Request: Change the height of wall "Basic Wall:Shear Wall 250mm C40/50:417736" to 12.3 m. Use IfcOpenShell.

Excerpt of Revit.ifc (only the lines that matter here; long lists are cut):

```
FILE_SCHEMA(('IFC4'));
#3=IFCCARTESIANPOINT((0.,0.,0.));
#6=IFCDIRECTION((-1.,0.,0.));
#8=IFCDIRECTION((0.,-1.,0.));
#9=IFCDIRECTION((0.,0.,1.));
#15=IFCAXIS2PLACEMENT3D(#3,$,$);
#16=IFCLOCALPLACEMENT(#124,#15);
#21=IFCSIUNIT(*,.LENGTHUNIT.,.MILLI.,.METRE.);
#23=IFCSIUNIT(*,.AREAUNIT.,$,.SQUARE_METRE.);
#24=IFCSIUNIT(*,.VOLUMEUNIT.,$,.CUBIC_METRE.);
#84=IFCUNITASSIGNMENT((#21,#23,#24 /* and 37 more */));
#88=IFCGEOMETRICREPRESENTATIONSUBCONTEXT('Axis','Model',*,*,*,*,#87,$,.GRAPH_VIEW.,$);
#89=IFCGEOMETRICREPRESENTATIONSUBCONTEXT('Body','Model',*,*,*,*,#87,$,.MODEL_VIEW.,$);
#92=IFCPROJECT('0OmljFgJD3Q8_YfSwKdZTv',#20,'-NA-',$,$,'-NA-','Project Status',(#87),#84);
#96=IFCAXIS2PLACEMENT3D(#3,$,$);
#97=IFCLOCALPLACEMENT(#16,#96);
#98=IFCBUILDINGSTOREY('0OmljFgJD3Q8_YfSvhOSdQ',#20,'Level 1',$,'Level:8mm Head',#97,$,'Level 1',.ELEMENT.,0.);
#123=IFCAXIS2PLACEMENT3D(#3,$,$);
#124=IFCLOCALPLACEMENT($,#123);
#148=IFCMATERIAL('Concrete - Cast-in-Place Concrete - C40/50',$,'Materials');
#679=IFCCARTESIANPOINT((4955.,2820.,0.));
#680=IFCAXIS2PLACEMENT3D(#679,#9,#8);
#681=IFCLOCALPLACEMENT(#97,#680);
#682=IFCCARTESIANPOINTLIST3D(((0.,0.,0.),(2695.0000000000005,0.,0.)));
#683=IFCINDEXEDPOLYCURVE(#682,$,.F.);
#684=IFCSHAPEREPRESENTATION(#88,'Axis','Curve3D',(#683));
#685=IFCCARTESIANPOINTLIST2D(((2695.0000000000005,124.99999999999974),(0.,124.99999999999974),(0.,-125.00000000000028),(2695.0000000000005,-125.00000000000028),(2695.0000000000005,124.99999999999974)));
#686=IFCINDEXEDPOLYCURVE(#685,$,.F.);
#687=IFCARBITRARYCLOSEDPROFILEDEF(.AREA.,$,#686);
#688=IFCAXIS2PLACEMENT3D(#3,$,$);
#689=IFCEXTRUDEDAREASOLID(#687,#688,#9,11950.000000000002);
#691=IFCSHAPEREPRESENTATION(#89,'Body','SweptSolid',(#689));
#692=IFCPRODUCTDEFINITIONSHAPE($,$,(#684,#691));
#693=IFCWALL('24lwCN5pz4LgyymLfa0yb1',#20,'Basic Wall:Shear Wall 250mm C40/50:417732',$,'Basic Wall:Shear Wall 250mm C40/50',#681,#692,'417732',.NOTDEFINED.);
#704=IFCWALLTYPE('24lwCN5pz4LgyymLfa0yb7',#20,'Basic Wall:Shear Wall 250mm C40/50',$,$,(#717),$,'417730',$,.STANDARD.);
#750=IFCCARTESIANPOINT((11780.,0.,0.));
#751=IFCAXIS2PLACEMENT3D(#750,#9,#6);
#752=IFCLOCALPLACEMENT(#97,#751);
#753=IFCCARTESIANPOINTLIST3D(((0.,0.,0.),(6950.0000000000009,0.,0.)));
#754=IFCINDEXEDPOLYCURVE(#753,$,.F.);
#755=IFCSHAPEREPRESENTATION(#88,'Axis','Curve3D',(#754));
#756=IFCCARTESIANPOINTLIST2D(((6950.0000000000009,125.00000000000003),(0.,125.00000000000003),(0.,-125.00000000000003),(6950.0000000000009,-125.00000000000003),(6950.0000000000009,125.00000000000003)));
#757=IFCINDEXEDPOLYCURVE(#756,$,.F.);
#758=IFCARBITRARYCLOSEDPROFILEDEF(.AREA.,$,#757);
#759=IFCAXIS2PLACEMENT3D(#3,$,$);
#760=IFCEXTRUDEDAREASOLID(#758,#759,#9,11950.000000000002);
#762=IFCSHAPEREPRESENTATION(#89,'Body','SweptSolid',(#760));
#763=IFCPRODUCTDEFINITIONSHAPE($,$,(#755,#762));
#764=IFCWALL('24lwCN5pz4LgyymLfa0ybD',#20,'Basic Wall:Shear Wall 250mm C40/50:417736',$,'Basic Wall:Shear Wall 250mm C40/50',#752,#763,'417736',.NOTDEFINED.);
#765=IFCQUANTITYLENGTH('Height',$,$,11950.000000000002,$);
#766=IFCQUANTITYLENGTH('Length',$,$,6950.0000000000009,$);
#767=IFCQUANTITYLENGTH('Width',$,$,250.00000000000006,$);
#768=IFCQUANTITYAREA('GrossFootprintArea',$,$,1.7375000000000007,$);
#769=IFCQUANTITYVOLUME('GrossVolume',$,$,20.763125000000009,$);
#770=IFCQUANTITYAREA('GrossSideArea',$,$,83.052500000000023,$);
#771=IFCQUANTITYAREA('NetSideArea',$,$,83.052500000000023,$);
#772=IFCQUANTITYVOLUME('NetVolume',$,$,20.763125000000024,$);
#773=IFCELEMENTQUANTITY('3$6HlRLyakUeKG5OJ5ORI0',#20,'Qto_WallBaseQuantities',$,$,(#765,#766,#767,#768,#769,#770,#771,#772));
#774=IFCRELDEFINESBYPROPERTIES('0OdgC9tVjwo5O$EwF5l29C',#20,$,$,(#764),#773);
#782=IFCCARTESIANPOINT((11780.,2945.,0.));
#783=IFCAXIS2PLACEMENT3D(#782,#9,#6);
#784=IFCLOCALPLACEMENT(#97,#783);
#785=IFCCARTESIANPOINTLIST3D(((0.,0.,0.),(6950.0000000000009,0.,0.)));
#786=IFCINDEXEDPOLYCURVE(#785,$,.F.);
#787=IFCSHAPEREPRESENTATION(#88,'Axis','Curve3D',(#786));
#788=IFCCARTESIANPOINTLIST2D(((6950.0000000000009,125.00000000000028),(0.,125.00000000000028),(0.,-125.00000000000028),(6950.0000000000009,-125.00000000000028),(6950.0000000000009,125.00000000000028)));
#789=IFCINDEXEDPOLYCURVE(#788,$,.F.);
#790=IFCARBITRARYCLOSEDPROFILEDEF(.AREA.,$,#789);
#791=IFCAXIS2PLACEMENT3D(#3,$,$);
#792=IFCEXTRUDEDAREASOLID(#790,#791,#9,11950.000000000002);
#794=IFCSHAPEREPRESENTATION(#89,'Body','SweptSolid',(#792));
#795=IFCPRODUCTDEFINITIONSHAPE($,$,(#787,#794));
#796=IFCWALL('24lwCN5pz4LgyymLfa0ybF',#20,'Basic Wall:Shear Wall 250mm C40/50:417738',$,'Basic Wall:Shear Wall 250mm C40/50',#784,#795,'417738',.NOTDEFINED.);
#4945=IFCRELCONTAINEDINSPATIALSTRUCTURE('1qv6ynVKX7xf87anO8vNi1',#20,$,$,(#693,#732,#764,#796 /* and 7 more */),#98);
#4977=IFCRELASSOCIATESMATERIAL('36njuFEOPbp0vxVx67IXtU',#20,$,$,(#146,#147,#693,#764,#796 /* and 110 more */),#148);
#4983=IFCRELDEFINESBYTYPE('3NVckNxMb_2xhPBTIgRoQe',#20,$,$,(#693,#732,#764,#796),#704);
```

```python
import ifcopenshell
import ifcopenshell.api.pset
import ifcopenshell.geom
import ifcopenshell.util.element
import ifcopenshell.util.representation
import ifcopenshell.util.shape
import ifcopenshell.util.unit

model = ifcopenshell.open("Revit.ifc")
unit_scale = ifcopenshell.util.unit.calculate_unit_scale(model)
area_scale = ifcopenshell.util.unit.calculate_unit_scale(model, "AREAUNIT")
volume_scale = ifcopenshell.util.unit.calculate_unit_scale(model, "VOLUMEUNIT")
settings = ifcopenshell.geom.settings()


def volume(element):
    """Net volume in cubic metres, openings subtracted."""
    shape = ifcopenshell.geom.create_shape(settings, element)
    return ifcopenshell.util.shape.get_volume(shape.geometry)


wall = model.by_guid("24lwCN5pz4LgyymLfa0ybD")
before = volume(wall)

body = ifcopenshell.util.representation.get_representation(wall, "Model", "Body")
solid = body.Items[0]
old_height = solid.Depth
solid.Depth = 12.3 / unit_scale
after = volume(wall)
thickness = 0.25  # wall thickness in metres

# Update the stored height, areas and volumes.
qto = model.by_id(ifcopenshell.util.element.get_pset(wall, "Qto_WallBaseQuantities", should_inherit=False)["id"])
ifcopenshell.api.pset.edit_qto(model, qto=qto, properties={
    "Height": solid.Depth,
    "GrossVolume": ifcopenshell.util.element.get_pset(wall, "Qto_WallBaseQuantities", "GrossVolume") * solid.Depth / old_height,
    "GrossSideArea": ifcopenshell.util.element.get_pset(wall, "Qto_WallBaseQuantities", "GrossSideArea") * solid.Depth / old_height,
    "NetSideArea": after / thickness / area_scale,
    "NetVolume": after / volume_scale,
})

print(f"height {old_height:g} -> {solid.Depth:g}, volume {before:.3f} -> {after:.3f} m3")

model.write("Revit-out.ifc")
```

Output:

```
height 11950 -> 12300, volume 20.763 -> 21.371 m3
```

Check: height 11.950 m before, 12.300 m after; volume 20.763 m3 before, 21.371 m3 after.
